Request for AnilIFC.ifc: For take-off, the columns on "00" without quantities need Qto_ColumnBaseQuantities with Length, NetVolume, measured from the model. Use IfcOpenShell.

First a look at what the model holds.

```python
import ifcopenshell
import ifcopenshell.util.element
import ifcopenshell.util.unit

model = ifcopenshell.open("AnilIFC.ifc")
print(model.schema)
for unit_type in ("LENGTHUNIT", "AREAUNIT", "VOLUMEUNIT"):
    print(unit_type, ifcopenshell.util.unit.calculate_unit_scale(model, unit_type))
storey = next(s for s in model.by_type("IfcBuildingStorey") if s.Name == "00")
columns = [e for e in ifcopenshell.util.element.get_decomposition(storey) if e.is_a("IfcColumn")]
for e in sorted(columns, key=lambda e: e.id()):
    print(e.id(), e.is_a(), e.Name, list(ifcopenshell.util.element.get_psets(e, qtos_only=True)), sep=" | ")
```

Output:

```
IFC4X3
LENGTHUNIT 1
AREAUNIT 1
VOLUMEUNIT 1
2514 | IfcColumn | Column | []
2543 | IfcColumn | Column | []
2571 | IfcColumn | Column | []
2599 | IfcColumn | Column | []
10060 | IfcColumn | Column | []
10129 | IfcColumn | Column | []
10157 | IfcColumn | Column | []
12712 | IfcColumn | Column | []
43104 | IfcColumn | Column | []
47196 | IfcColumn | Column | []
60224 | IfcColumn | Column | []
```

```python
import ifcopenshell
import ifcopenshell.api.pset
import ifcopenshell.geom
import ifcopenshell.util.element
import ifcopenshell.util.shape
import ifcopenshell.util.unit

model = ifcopenshell.open("AnilIFC.ifc")
unit_scale = ifcopenshell.util.unit.calculate_unit_scale(model)
volume_scale = ifcopenshell.util.unit.calculate_unit_scale(model, "VOLUMEUNIT")
settings = ifcopenshell.geom.settings()

storey = next(s for s in model.by_type("IfcBuildingStorey") if s.Name == "00")
columns = [e for e in ifcopenshell.util.element.get_decomposition(storey) if e.is_a("IfcColumn")]

for e in sorted(columns, key=lambda e: e.id()):
    if ifcopenshell.util.element.get_psets(e, qtos_only=True, should_inherit=False):
        continue
    # Geometry comes back in metres, in the element's own axes.
    shape = ifcopenshell.geom.create_shape(settings, e)
    values = {
        "Length": ifcopenshell.util.shape.get_z(shape.geometry) / unit_scale,
        "NetVolume": ifcopenshell.util.shape.get_volume(shape.geometry) / volume_scale,
    }
    qto = ifcopenshell.api.pset.add_qto(model, product=e, name="Qto_ColumnBaseQuantities")
    ifcopenshell.api.pset.edit_qto(model, qto=qto, properties=values)
    print(e.id(), {k: round(v, 3) for k, v in values.items()})

model.write("AnilIFC_edited.ifc")
```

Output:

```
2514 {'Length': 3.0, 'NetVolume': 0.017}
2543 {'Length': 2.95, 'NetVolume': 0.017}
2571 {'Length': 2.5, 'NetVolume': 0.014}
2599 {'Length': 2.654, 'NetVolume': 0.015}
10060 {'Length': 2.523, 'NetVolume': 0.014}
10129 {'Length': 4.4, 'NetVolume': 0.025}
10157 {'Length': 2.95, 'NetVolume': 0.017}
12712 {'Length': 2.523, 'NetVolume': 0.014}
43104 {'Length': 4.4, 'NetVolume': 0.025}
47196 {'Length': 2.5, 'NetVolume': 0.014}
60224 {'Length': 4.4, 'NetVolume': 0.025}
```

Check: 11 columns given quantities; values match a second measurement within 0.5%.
